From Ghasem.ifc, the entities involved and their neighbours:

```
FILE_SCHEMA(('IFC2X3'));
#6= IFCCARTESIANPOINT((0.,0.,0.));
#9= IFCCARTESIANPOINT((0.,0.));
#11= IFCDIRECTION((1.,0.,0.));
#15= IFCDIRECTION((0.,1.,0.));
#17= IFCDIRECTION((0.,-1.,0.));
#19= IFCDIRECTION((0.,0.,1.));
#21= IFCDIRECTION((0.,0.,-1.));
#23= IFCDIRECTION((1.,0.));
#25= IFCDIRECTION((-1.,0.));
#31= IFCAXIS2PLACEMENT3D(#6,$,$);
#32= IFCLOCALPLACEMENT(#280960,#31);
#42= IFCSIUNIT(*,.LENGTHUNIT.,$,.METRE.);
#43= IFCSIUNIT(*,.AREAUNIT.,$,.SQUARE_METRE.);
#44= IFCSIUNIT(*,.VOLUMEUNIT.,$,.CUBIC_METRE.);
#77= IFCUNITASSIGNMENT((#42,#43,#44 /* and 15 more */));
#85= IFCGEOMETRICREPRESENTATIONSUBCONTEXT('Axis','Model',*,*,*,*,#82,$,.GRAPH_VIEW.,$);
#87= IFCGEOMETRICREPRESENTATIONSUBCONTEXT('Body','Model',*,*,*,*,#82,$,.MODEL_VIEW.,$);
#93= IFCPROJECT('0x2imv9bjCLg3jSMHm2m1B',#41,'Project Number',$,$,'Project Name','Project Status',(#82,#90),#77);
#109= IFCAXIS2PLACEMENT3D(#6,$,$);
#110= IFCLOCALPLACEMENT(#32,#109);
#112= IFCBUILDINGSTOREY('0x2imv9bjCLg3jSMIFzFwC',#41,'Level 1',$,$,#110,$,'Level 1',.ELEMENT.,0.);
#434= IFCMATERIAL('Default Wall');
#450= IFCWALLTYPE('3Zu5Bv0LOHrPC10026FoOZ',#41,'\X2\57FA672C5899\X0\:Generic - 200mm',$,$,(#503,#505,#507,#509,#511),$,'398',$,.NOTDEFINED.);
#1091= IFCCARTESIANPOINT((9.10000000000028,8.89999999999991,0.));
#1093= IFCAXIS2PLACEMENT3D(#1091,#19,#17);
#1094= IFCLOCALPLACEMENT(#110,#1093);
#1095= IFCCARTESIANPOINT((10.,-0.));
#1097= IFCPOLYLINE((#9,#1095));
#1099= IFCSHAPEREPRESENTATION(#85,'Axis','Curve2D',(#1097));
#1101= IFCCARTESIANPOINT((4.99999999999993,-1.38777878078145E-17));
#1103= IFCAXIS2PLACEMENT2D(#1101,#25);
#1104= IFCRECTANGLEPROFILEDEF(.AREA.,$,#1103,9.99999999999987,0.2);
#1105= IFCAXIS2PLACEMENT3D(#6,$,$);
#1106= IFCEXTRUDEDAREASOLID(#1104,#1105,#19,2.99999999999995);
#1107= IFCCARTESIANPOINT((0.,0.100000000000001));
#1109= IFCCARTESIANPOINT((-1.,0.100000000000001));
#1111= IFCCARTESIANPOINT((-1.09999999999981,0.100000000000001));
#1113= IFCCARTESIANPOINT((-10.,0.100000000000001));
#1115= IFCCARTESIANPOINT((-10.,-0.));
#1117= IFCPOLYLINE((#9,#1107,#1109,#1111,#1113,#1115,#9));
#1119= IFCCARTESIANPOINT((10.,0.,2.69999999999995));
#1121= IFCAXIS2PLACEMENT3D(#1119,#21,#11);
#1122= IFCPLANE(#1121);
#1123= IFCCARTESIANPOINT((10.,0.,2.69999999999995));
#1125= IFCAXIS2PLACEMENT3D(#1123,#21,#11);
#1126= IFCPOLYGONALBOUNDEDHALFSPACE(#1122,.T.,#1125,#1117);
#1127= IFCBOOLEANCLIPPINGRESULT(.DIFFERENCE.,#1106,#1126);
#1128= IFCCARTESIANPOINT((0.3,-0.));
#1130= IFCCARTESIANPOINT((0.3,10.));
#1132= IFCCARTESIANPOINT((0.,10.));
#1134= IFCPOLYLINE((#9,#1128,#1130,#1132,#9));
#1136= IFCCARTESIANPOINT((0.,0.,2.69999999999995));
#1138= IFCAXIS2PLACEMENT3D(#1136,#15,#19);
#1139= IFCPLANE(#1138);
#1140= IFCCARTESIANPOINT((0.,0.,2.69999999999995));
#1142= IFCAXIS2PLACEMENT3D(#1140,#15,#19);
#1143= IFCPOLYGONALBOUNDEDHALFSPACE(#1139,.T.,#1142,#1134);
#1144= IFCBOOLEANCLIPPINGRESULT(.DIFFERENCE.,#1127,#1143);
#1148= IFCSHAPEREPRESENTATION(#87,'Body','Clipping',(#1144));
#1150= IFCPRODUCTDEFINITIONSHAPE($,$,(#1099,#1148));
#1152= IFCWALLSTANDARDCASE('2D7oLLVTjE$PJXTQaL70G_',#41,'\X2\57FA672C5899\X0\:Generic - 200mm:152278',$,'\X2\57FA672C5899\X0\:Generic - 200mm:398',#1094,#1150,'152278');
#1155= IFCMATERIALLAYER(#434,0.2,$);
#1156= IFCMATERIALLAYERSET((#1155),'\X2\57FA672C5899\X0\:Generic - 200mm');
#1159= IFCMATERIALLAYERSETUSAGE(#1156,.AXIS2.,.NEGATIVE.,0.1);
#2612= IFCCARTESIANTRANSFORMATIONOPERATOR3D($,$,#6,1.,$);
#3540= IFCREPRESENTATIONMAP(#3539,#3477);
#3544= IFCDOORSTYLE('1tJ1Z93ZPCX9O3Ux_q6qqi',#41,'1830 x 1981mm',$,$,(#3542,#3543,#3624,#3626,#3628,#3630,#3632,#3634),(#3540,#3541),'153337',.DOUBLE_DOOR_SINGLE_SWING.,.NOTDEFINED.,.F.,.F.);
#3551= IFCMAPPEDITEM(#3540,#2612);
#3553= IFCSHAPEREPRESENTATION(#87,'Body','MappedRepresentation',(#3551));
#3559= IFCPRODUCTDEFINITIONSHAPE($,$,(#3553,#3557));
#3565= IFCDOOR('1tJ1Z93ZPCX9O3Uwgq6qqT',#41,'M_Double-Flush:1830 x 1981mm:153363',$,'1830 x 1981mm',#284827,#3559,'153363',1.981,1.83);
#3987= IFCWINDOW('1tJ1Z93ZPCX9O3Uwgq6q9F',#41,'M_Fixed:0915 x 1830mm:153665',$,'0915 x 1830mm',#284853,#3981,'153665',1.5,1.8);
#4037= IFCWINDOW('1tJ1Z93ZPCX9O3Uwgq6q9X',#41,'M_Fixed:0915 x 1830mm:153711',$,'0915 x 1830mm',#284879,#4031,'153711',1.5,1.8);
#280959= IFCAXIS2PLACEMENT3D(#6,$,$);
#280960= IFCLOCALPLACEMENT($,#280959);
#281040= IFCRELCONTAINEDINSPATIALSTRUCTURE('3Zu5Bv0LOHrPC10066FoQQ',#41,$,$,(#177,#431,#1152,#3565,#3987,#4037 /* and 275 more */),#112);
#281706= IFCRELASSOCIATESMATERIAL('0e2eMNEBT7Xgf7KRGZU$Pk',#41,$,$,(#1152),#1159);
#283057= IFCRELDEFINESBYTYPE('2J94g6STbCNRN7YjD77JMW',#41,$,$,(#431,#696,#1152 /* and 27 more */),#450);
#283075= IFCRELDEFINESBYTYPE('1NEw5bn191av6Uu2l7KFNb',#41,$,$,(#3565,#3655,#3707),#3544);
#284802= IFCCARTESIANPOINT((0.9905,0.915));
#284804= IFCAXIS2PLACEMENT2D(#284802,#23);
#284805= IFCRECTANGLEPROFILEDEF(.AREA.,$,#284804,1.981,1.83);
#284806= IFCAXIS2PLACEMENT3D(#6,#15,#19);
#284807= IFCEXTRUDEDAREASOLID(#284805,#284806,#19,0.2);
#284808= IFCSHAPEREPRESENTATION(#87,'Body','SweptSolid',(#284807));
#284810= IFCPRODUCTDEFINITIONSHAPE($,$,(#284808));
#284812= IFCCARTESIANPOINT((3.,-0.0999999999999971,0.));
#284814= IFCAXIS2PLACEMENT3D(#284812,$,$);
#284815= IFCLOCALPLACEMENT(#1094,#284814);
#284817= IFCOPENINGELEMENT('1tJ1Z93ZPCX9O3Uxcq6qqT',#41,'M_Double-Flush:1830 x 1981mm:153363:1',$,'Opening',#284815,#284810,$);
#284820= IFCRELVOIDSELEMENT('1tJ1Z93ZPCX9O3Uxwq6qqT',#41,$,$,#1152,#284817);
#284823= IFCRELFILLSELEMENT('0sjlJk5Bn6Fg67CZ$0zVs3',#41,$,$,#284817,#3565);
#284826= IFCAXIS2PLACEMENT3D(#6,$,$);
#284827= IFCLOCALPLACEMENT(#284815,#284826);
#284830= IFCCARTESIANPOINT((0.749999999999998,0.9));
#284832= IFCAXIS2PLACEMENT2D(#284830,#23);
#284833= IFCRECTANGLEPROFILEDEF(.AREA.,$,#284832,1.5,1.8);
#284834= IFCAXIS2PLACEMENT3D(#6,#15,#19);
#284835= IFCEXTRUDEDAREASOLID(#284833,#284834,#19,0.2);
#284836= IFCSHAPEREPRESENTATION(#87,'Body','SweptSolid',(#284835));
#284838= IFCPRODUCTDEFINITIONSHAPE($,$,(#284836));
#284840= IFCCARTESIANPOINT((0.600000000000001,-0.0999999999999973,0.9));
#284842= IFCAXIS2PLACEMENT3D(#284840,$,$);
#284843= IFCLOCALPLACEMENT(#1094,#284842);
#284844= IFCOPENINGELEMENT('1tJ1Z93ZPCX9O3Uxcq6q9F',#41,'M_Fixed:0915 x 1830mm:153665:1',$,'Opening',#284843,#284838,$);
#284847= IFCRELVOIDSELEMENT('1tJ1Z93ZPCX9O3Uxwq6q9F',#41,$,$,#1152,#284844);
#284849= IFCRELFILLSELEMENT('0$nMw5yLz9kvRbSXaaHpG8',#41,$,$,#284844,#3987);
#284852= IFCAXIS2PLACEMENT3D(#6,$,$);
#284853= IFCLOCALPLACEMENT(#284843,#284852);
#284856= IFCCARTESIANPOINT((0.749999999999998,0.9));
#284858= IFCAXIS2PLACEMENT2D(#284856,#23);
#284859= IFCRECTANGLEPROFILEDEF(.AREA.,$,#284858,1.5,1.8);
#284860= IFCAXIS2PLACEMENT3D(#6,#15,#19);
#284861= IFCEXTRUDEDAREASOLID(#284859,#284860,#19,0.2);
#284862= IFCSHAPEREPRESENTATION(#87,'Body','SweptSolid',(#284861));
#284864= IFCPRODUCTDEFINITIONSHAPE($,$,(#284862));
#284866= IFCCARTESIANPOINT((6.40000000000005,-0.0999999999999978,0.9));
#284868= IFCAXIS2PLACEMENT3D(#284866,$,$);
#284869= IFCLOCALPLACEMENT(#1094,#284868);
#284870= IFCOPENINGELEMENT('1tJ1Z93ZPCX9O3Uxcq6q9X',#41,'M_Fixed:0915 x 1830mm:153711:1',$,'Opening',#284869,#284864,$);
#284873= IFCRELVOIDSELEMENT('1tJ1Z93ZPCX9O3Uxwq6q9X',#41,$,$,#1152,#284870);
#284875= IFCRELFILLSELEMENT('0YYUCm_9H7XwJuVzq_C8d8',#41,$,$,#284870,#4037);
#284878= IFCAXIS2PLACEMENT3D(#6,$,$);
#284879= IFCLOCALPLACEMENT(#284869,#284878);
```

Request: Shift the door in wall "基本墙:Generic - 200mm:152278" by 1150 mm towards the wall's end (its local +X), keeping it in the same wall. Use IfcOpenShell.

```python
import ifcopenshell
import ifcopenshell.api.geometry
import ifcopenshell.util.placement
import ifcopenshell.util.unit

model = ifcopenshell.open("Ghasem.ifc")
unit_scale = ifcopenshell.util.unit.calculate_unit_scale(model)

door = model.by_guid("1tJ1Z93ZPCX9O3Uwgq6qqT")
opening = door.FillsVoids[0].RelatingOpeningElement
wall = opening.VoidsElements[0].RelatingBuildingElement

wall_matrix = ifcopenshell.util.placement.get_local_placement(wall.ObjectPlacement)
shift = wall_matrix[:3, 0] * 1.15 / unit_scale
before = ifcopenshell.util.placement.get_local_placement(door.ObjectPlacement)[:3, 3].copy()

# The door is placed relative to its opening, so it follows when the opening moves.
matrix = ifcopenshell.util.placement.get_local_placement(opening.ObjectPlacement)
matrix[:3, 3] += shift
ifcopenshell.api.geometry.edit_object_placement(
    model, product=opening, matrix=matrix, is_si=False, should_transform_children=True
)

after = ifcopenshell.util.placement.get_local_placement(door.ObjectPlacement)[:3, 3]
print("door moved by", (after - before).round(3) + 0.0)

model.write("Ghasem-out.ifc")
```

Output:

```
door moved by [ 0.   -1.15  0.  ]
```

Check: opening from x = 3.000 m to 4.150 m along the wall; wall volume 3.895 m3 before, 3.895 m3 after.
